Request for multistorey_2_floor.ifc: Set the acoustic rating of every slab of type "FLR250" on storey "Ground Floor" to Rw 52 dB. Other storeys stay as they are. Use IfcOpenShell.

First a look at what the model holds.

```python
import ifcopenshell
import ifcopenshell.util.element

model = ifcopenshell.open("multistorey_2_floor.ifc")
print(model.schema)
storey = next(s for s in model.by_type("IfcBuildingStorey") if s.Name == "Ground Floor")
slabs = [e for e in ifcopenshell.util.element.get_decomposition(storey) if e.is_a("IfcSlab")]
seen = {}
for e in slabs:
    element_type = ifcopenshell.util.element.get_type(e)
    key = (element_type.Name if element_type != e and element_type else None, ifcopenshell.util.element.get_pset(e, "Pset_SlabCommon", "AcousticRating"))
    seen[key] = seen.get(key, 0) + 1
for (name, value), count in sorted(seen.items(), key=str):
    print(count, "x", name, "|", value)
```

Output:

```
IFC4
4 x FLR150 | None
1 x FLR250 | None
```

```python
import ifcopenshell
import ifcopenshell.api.pset
import ifcopenshell.util.element

model = ifcopenshell.open("multistorey_2_floor.ifc")

storey = next(s for s in model.by_type("IfcBuildingStorey") if s.Name == "Ground Floor")
slabs = [e for e in ifcopenshell.util.element.get_decomposition(storey) if e.is_a("IfcSlab")]

count = 0
for e in slabs:
    element_type = ifcopenshell.util.element.get_type(e)
    if element_type in (None, e) or element_type.Name != "FLR250":
        continue
    # add_pset returns the element's existing set when there is one.
    pset = ifcopenshell.api.pset.add_pset(model, product=e, name="Pset_SlabCommon")
    ifcopenshell.api.pset.edit_pset(model, pset=pset, properties={"AcousticRating": "Rw 52 dB"})
    count += 1

print(count, "slabs updated")

model.write("multistorey_2_floor_updated.ifc")
```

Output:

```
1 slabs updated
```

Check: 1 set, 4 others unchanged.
